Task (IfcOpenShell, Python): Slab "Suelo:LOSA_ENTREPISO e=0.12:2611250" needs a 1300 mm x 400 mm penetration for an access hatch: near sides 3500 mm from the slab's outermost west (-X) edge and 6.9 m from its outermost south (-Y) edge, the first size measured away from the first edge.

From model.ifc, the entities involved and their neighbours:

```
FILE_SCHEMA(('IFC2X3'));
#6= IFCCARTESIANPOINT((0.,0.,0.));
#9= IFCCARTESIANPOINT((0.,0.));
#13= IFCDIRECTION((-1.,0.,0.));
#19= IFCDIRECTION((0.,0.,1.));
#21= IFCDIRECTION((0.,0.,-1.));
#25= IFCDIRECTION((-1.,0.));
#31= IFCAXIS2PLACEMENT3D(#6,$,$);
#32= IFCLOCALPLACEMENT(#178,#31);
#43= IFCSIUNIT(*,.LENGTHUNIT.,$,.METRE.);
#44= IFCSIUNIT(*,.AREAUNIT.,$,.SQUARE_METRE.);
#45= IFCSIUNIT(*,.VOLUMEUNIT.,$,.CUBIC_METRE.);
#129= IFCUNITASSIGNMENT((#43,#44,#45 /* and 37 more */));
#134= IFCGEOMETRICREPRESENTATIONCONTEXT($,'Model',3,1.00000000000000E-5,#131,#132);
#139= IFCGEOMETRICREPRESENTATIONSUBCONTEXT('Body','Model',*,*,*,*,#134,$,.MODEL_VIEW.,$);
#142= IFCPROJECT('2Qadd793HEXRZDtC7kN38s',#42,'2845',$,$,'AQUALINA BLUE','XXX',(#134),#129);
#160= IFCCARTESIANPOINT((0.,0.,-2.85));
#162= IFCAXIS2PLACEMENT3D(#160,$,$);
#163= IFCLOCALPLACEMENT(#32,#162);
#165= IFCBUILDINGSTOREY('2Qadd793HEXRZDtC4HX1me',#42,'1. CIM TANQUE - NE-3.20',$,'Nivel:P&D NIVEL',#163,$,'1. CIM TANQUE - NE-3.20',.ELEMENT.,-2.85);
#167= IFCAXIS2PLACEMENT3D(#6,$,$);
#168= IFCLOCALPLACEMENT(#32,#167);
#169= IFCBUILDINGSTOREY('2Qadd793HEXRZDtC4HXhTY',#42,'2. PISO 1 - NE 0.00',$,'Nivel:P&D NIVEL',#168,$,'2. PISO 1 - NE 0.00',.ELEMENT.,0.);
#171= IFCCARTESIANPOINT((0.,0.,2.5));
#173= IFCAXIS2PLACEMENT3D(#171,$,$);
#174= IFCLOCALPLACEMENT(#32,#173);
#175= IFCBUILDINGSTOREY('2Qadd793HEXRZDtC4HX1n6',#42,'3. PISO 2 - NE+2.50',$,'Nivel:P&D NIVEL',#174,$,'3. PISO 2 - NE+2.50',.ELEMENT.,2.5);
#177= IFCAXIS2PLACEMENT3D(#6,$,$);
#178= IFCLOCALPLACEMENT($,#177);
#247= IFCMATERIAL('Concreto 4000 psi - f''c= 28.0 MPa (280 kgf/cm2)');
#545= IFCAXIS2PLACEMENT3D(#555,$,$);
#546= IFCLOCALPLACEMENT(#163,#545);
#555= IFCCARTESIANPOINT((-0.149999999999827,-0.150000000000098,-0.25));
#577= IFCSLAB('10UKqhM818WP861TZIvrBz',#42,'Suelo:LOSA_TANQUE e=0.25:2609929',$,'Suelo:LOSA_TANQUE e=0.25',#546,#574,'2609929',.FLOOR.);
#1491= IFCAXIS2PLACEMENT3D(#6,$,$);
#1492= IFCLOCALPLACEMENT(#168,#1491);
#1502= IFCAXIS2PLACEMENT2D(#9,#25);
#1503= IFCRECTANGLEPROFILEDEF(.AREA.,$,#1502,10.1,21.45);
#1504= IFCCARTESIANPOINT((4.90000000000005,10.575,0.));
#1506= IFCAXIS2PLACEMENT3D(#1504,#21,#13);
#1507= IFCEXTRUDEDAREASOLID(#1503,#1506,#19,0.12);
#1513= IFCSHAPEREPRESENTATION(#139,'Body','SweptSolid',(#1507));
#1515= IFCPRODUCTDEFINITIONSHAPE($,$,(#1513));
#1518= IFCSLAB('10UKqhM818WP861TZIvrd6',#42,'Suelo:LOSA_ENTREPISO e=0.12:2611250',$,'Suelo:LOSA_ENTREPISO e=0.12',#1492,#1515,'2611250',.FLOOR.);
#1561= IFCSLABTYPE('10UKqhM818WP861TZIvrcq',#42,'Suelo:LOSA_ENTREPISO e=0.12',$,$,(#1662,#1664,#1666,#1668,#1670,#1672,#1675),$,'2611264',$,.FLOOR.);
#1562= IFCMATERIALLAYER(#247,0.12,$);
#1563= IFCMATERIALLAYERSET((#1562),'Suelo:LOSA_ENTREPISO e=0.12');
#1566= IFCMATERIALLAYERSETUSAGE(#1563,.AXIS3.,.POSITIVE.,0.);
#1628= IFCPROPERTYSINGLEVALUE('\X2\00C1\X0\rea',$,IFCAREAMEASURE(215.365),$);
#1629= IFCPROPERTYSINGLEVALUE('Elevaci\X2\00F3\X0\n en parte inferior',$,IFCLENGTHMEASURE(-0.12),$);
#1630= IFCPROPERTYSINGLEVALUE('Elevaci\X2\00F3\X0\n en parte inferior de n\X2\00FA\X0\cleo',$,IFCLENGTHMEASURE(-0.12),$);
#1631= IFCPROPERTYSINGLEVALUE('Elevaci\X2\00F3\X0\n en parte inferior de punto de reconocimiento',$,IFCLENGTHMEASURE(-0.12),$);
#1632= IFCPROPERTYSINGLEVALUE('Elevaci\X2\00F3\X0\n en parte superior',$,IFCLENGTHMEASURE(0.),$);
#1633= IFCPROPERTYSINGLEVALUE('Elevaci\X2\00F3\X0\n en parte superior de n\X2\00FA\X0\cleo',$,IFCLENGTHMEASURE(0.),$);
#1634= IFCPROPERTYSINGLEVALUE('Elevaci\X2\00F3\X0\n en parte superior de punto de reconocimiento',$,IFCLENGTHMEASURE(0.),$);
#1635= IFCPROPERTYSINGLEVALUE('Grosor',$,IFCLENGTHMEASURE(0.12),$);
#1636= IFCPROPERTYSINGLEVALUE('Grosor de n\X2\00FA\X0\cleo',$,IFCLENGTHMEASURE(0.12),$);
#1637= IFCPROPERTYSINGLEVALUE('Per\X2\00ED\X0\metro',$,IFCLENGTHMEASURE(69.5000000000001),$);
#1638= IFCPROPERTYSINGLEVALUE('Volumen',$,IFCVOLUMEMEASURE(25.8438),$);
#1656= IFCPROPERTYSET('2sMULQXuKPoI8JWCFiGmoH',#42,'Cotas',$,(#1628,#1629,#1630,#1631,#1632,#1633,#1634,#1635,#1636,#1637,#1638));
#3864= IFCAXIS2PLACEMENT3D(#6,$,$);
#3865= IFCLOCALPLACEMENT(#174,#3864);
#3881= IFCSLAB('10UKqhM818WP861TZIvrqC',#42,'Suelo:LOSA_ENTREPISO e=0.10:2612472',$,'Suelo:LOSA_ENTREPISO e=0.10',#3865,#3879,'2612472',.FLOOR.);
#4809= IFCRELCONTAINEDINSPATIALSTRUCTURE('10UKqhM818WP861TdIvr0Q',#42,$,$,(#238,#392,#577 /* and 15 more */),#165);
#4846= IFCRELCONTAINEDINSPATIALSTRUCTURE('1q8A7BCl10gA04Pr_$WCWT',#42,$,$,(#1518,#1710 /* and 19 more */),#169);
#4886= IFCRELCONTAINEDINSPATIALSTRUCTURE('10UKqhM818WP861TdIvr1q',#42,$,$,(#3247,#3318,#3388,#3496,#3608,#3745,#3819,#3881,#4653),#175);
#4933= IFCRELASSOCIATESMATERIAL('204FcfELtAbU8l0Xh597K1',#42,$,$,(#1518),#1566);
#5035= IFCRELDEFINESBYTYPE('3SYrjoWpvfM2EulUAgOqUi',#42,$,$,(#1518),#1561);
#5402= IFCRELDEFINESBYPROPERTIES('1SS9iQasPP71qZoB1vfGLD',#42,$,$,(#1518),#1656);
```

```python
import numpy as np
import ifcopenshell
import ifcopenshell.api.feature
import ifcopenshell.api.geometry
import ifcopenshell.api.pset
import ifcopenshell.api.root
import ifcopenshell.geom
import ifcopenshell.util.element
import ifcopenshell.util.placement
import ifcopenshell.util.representation
import ifcopenshell.util.shape
import ifcopenshell.util.unit

model = ifcopenshell.open("model.ifc")
unit_scale = ifcopenshell.util.unit.calculate_unit_scale(model)
area_scale = ifcopenshell.util.unit.calculate_unit_scale(model, "AREAUNIT")
volume_scale = ifcopenshell.util.unit.calculate_unit_scale(model, "VOLUMEUNIT")
settings = ifcopenshell.geom.settings()


def volume(element):
    """Net volume in cubic metres, openings subtracted."""
    shape = ifcopenshell.geom.create_shape(settings, element)
    return ifcopenshell.util.shape.get_volume(shape.geometry)


slab = model.by_guid("10UKqhM818WP861TZIvrd6")
before = volume(slab)

# Extent in the slab's own axes, in metres. The edges named are its -X and -Y sides.
slab_shape = ifcopenshell.geom.create_shape(settings, slab)
vertices = ifcopenshell.util.shape.get_vertices(slab_shape.geometry)
x_min, y_min, bottom = vertices.min(axis=0)
top = vertices[:, 2].max()

opening = ifcopenshell.api.root.create_entity(model, ifc_class="IfcOpeningElement", name="Access hatch opening")
context = ifcopenshell.util.representation.get_context(model, "Model", "Body", "MODEL_VIEW")
width, depth = 1.3, 0.4
outline = [(0.0, 0.0), (width, 0.0), (width, depth), (0.0, depth), (0.0, 0.0)]
# Overshoot both faces by 50 mm so the cut is clean.
shape = ifcopenshell.api.geometry.add_slab_representation(
    model, context=context, depth=top - bottom + 0.1, polyline=outline
)
ifcopenshell.api.geometry.assign_representation(model, product=opening, representation=shape)

matrix = ifcopenshell.util.placement.get_local_placement(slab.ObjectPlacement)
matrix[:, 3] = matrix @ np.append(np.array([x_min + 3.5, y_min + 6.9, bottom - 0.05]) / unit_scale, 1.0)
ifcopenshell.api.geometry.edit_object_placement(model, product=opening, matrix=matrix, is_si=False)
ifcopenshell.api.feature.add_feature(model, feature=opening, element=slab)

after = volume(slab)

# Update the slab's stored quantities.
pset = model.by_id(ifcopenshell.util.element.get_pset(slab, "Cotas", should_inherit=False)["id"])
ifcopenshell.api.pset.edit_pset(model, pset=pset, properties={
    "Área": model.create_entity("IfcAreaMeasure", after / (top - bottom) / area_scale),
    "Volumen": model.create_entity("IfcVolumeMeasure", after / volume_scale),
})

print(f"slab volume {before:.3f} -> {after:.3f} m3")

model.write("model_rev.ifc")
```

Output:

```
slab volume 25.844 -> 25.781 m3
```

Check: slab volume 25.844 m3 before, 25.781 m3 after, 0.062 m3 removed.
